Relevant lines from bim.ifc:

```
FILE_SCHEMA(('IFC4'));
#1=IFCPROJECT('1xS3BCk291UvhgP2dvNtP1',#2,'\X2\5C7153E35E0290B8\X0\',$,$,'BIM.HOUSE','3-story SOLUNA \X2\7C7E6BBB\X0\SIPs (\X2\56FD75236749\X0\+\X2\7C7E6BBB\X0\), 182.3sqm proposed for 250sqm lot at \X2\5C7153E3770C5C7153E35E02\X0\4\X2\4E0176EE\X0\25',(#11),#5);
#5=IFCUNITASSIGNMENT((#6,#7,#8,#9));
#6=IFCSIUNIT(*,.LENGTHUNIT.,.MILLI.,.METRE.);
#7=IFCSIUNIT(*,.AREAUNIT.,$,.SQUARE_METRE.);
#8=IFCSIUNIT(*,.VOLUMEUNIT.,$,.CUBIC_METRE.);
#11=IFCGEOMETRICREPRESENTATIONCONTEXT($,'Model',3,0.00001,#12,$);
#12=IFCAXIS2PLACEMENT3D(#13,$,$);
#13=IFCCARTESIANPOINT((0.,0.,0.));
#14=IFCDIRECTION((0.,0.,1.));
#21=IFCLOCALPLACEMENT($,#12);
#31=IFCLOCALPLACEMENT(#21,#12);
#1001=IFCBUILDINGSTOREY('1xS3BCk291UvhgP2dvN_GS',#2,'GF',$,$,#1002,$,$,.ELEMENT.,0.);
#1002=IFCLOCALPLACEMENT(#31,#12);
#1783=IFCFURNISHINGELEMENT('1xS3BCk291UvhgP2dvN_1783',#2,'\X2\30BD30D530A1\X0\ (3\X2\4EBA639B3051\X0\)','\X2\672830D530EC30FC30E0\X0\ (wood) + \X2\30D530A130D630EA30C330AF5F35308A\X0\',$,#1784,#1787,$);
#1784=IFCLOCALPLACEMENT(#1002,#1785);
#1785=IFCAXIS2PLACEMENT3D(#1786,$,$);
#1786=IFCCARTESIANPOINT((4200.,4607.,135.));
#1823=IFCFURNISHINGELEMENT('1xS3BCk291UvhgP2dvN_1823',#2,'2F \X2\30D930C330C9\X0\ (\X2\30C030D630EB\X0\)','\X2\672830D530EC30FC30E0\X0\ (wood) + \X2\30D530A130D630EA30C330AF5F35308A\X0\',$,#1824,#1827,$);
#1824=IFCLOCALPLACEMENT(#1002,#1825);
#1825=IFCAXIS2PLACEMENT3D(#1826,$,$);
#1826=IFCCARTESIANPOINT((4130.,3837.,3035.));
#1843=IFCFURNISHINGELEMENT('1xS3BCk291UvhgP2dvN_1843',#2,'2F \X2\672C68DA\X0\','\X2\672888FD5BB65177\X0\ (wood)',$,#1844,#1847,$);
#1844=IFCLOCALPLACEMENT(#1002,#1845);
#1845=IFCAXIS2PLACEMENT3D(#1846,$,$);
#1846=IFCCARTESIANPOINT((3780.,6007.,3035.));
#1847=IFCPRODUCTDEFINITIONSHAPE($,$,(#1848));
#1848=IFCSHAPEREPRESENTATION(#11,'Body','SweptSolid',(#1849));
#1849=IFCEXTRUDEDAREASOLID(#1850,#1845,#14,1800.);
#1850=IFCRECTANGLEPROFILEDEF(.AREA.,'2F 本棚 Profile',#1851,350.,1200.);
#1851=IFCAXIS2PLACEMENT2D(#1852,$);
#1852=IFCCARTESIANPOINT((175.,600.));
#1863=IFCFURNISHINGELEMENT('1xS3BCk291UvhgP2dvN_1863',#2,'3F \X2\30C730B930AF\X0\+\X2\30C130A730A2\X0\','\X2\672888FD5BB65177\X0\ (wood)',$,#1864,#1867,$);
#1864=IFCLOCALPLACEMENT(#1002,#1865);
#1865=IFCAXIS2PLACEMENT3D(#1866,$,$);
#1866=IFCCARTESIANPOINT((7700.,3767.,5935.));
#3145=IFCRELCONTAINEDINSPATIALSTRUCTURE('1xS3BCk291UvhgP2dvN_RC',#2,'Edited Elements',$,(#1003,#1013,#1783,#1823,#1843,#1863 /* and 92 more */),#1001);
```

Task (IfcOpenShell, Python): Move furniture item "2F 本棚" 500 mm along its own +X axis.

```python
import ifcopenshell
import ifcopenshell.api.geometry
import ifcopenshell.util.placement

model = ifcopenshell.open("bim.ifc")

item = model.by_guid("1xS3BCk291UvhgP2dvN_1843")
matrix = ifcopenshell.util.placement.get_local_placement(item.ObjectPlacement)
matrix[:3, 3] += matrix[:3, 0] * 500.0
ifcopenshell.api.geometry.edit_object_placement(model, product=item, matrix=matrix, is_si=False)

print(ifcopenshell.util.placement.get_local_placement(item.ObjectPlacement).round(3) + 0.0)

model.write("bim_rev.ifc")
```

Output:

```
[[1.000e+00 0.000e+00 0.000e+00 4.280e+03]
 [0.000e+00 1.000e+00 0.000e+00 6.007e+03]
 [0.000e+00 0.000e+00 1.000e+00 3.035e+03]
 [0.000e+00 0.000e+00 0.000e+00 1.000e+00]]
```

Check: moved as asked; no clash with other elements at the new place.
